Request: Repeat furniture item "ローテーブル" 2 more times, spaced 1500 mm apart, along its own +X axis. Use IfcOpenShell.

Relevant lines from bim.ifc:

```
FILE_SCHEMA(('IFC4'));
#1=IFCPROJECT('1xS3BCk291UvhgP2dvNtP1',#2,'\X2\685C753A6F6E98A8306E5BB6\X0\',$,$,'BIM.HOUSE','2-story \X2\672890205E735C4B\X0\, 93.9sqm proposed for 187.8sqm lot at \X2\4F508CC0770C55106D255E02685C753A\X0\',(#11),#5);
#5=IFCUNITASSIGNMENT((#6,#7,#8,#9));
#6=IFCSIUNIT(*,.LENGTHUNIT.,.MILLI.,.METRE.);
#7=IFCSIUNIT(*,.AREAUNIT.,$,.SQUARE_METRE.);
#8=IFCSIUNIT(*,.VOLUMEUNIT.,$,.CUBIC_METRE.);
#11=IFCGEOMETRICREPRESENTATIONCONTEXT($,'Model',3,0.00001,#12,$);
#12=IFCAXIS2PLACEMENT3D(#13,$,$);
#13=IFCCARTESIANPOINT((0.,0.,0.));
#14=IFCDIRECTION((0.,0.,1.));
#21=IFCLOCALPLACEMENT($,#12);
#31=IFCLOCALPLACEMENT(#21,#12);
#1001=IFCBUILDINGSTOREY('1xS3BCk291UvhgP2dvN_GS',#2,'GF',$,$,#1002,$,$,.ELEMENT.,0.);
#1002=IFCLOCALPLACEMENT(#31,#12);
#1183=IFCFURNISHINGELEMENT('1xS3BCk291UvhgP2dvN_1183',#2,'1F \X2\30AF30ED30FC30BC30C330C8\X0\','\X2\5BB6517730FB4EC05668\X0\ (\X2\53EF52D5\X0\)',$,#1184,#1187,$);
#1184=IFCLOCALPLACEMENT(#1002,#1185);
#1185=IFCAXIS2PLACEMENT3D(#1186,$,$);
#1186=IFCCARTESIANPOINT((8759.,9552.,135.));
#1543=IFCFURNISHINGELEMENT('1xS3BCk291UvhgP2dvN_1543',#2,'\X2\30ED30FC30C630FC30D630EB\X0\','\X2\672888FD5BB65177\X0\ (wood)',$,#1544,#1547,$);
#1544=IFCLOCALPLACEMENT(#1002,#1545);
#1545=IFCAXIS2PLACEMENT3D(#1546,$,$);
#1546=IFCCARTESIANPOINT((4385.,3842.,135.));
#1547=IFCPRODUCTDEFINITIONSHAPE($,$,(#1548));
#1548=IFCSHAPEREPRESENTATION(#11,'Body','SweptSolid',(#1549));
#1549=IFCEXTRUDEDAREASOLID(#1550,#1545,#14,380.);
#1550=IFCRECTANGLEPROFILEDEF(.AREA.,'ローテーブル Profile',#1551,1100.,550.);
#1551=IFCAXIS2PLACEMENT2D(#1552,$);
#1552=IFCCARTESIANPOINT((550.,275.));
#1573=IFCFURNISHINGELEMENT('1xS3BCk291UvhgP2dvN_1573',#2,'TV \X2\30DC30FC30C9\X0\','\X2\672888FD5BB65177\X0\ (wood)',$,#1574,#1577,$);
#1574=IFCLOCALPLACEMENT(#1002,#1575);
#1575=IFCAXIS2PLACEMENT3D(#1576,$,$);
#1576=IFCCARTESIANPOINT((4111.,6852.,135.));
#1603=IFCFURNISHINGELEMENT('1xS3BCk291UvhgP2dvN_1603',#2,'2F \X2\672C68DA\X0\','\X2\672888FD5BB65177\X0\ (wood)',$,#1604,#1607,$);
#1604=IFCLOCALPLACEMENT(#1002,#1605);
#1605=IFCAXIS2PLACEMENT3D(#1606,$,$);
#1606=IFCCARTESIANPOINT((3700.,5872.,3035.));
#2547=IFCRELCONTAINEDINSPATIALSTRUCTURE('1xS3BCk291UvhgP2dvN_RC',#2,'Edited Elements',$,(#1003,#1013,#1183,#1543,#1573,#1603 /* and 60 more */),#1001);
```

```python
import ifcopenshell
import ifcopenshell.api.geometry
import ifcopenshell.api.root
import ifcopenshell.util.element
import ifcopenshell.util.placement
import ifcopenshell.util.unit

model = ifcopenshell.open("bim.ifc")
unit_scale = ifcopenshell.util.unit.calculate_unit_scale(model)


def reuse_history(source, copy):
    """copy_class also copies each property set's owner history, people and application; keep the originals."""
    for rel in copy.IsDefinedBy:
        if rel.is_a("IfcRelDefinesByProperties") and (history := rel.RelatingPropertyDefinition.OwnerHistory):
            rel.RelatingPropertyDefinition.OwnerHistory = source.OwnerHistory
            ifcopenshell.util.element.remove_deep2(model, history)


source = model.by_guid("1xS3BCk291UvhgP2dvN_1543")
base = ifcopenshell.util.placement.get_local_placement(source.ObjectPlacement)
step = base[:3, 0] * 1.5 / unit_scale

for i in range(1, 3):
    copy = ifcopenshell.api.root.copy_class(model, product=source)
    copy.Representation = ifcopenshell.util.element.copy_deep(
        model, source.Representation, exclude=["IfcGeometricRepresentationContext", "IfcRepresentationMap"]
    )
    reuse_history(source, copy)
    matrix = base.copy()
    matrix[:3, 3] += i * step
    print("added at", matrix[:3, 3].round(3) + 0.0)
    ifcopenshell.api.geometry.edit_object_placement(model, product=copy, matrix=matrix, is_si=False)

model.write("bim-out.ifc")
```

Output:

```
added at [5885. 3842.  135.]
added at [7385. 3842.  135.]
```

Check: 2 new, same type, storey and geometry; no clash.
